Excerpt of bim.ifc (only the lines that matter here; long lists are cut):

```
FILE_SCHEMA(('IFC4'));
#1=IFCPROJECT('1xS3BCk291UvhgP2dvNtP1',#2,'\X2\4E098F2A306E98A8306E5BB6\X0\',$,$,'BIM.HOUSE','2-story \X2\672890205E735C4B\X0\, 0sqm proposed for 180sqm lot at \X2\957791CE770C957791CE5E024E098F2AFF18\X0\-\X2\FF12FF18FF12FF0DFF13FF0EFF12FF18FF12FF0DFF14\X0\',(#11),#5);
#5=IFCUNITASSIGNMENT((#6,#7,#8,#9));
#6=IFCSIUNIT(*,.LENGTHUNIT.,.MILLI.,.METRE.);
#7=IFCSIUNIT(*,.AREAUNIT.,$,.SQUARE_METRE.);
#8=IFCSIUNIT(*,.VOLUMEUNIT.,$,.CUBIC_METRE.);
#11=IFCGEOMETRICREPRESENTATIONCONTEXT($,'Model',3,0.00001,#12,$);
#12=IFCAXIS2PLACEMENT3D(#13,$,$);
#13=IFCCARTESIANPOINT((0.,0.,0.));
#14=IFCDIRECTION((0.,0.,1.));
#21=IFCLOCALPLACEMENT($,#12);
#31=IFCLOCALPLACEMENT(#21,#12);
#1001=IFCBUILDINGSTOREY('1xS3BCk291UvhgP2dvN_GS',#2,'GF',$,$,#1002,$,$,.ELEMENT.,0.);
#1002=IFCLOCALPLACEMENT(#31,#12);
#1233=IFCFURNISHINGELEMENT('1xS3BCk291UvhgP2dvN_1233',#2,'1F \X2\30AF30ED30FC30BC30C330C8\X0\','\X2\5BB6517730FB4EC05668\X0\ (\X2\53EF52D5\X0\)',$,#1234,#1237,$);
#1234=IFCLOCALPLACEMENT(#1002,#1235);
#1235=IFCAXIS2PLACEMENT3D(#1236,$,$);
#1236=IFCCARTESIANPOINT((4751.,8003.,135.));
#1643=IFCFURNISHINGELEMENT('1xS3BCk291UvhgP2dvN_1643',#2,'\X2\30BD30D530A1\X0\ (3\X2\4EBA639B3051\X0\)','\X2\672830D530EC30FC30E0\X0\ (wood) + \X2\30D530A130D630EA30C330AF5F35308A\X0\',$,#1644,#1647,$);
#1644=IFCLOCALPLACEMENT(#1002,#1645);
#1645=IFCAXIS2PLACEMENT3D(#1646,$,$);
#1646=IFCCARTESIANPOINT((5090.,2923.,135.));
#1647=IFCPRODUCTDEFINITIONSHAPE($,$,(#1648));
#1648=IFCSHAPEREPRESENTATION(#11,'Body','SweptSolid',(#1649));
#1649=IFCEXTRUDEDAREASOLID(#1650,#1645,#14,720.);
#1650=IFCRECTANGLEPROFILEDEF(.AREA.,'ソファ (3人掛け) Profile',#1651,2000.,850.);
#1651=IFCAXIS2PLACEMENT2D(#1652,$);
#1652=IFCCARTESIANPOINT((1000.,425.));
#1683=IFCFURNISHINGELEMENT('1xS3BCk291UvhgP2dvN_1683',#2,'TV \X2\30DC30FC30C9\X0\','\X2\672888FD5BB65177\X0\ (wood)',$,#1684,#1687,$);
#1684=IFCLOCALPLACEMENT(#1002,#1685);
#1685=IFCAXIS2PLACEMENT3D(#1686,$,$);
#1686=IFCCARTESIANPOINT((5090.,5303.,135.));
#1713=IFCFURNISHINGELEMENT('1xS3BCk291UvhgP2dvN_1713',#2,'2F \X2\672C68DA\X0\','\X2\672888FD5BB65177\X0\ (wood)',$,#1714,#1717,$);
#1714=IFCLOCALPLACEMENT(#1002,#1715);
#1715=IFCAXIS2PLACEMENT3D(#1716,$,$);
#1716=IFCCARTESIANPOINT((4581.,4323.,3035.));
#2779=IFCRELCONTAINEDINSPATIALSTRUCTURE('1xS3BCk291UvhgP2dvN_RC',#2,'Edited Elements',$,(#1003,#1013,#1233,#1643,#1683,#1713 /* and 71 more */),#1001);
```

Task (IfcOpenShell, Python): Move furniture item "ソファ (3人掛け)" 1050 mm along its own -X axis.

```python
import ifcopenshell
import ifcopenshell.api.geometry
import ifcopenshell.util.placement

model = ifcopenshell.open("bim.ifc")

item = model.by_guid("1xS3BCk291UvhgP2dvN_1643")
matrix = ifcopenshell.util.placement.get_local_placement(item.ObjectPlacement)
matrix[:3, 3] -= matrix[:3, 0] * 1050.0
ifcopenshell.api.geometry.edit_object_placement(model, product=item, matrix=matrix, is_si=False)

print(ifcopenshell.util.placement.get_local_placement(item.ObjectPlacement).round(3) + 0.0)

model.write("bim_edited.ifc")
```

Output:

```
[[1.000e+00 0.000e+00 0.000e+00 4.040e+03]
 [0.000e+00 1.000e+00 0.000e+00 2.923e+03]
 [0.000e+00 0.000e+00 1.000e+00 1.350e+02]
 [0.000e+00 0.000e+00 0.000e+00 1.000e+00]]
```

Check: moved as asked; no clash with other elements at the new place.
